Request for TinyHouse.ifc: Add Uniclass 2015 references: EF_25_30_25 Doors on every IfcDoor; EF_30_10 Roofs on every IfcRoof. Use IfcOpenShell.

First a look at what the model holds.

```python
import ifcopenshell

model = ifcopenshell.open("TinyHouse.ifc")
print(model.schema)
print("classifications:", [c.Name for c in model.by_type("IfcClassification")])
for ifc_class in ("IfcDoor", "IfcRoof", "IfcStair", "IfcWall", "IfcWindow"):
    print(ifc_class, len(model.by_type(ifc_class)))
```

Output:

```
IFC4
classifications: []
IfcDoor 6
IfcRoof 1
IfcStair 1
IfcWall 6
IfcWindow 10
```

```python
import ifcopenshell
import ifcopenshell.api.classification

model = ifcopenshell.open("TinyHouse.ifc")

system = ifcopenshell.api.classification.add_classification(model, classification="Uniclass 2015")

codes = {
    "IfcDoor": ("EF_25_30_25", "Doors"),
    "IfcRoof": ("EF_30_10", "Roofs"),
}
for ifc_class, (code, name) in codes.items():
    products = model.by_type(ifc_class)
    ifcopenshell.api.classification.add_reference(
        model, products=products, classification=system, identification=code, name=name
    )
    print(code, len(products))

model.write("TinyHouse_rev.ifc")
```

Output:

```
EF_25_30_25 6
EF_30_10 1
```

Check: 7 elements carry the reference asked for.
